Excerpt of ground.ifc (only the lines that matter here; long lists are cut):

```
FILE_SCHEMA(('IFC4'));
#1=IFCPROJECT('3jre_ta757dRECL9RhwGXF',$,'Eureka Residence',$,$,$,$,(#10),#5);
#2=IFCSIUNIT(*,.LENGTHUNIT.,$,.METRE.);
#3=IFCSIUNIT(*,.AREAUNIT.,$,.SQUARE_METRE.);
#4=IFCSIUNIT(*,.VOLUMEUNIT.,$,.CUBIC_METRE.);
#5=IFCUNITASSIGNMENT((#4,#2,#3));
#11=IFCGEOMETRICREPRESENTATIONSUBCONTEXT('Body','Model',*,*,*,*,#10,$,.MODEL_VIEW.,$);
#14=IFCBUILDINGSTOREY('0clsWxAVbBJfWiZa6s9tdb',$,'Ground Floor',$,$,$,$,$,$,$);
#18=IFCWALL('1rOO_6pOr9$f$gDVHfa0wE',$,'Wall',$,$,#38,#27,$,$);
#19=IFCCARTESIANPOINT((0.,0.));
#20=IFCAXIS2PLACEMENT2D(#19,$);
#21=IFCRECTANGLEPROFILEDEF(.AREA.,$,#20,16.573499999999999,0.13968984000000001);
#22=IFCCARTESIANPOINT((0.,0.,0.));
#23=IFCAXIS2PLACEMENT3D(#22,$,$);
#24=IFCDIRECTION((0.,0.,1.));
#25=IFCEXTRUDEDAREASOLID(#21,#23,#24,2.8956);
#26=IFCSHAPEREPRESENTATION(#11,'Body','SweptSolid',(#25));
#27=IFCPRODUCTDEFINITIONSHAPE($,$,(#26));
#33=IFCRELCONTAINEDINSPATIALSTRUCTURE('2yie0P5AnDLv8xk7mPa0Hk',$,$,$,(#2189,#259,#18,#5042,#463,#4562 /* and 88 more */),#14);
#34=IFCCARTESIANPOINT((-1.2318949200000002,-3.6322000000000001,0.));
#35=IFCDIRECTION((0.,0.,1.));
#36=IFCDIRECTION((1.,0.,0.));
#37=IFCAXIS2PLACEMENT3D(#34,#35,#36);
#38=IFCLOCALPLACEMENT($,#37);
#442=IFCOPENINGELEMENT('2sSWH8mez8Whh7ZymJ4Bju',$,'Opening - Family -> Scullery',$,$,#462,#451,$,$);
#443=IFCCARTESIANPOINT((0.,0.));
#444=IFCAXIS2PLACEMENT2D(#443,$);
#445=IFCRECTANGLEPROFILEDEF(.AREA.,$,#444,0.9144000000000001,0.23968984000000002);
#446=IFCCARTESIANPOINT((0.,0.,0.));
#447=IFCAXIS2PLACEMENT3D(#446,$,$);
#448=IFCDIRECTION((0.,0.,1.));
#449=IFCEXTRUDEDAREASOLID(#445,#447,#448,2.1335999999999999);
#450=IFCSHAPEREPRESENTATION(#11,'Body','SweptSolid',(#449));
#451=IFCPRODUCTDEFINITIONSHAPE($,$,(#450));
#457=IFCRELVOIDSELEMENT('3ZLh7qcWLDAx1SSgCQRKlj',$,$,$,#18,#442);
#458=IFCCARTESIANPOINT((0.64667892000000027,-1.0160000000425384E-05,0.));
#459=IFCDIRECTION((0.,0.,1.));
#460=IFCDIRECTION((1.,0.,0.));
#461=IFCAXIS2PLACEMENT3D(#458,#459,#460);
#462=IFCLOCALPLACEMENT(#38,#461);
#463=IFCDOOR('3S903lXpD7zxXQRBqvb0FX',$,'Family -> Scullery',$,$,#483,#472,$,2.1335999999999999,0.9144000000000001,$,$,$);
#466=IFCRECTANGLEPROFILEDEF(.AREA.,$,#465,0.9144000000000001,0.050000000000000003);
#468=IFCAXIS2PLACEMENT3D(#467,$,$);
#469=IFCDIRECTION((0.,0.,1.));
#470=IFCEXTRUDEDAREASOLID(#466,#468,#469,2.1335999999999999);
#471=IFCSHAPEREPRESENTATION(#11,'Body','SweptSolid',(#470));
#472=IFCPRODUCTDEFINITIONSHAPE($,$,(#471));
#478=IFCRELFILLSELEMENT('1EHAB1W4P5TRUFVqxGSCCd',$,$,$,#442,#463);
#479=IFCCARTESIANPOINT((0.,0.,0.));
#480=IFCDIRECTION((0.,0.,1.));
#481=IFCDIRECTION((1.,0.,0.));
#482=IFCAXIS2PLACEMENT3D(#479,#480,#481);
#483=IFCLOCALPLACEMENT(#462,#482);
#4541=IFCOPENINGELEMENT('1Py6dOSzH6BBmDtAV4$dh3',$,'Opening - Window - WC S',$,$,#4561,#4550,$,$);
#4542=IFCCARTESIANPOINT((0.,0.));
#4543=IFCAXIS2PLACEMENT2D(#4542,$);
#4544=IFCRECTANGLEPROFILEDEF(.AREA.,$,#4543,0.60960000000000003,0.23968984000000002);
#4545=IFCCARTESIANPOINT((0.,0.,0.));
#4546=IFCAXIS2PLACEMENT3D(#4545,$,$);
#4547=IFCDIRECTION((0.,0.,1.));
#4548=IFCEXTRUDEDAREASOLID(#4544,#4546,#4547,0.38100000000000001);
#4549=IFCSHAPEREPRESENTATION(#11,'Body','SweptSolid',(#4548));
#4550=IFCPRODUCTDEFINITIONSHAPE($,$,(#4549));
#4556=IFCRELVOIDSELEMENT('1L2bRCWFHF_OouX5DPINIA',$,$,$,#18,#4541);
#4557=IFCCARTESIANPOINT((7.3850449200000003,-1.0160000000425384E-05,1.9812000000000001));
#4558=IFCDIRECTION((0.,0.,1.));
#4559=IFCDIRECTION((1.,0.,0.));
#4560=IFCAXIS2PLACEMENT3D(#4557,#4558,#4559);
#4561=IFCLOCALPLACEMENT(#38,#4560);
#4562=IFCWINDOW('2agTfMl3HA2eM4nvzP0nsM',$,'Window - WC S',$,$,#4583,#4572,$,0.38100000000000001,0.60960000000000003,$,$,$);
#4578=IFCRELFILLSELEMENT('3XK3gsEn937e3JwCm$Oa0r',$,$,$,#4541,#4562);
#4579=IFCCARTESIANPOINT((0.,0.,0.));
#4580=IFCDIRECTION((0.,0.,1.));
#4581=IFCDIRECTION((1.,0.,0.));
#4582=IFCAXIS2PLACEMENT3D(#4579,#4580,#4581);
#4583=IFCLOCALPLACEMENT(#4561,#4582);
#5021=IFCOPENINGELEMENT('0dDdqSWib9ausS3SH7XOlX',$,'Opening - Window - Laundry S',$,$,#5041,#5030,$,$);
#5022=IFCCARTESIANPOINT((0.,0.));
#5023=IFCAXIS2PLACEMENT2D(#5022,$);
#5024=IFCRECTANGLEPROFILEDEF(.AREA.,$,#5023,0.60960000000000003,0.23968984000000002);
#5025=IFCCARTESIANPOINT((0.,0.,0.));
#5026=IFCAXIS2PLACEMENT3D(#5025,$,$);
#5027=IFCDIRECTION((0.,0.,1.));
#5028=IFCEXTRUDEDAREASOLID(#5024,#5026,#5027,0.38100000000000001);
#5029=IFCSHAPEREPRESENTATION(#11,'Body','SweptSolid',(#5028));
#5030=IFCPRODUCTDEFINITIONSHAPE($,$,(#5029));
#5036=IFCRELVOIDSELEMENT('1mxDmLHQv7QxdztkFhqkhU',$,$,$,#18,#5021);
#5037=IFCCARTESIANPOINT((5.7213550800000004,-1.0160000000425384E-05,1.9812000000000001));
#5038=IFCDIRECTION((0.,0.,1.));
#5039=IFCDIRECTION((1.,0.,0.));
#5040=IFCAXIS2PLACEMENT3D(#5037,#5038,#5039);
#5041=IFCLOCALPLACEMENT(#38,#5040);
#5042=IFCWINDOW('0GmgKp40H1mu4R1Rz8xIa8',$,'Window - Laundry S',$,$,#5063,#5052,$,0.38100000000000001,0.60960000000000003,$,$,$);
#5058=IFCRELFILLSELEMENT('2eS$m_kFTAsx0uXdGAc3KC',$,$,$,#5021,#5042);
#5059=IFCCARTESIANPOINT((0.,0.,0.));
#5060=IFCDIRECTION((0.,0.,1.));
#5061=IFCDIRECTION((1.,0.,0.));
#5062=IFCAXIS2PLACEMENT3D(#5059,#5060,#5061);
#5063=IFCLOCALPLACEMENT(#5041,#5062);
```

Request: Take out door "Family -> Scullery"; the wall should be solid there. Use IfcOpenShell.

```python
import ifcopenshell
import ifcopenshell.api.feature
import ifcopenshell.api.root
import ifcopenshell.geom
import ifcopenshell.util.shape

model = ifcopenshell.open("ground.ifc")
settings = ifcopenshell.geom.settings()


def volume(element):
    """Net volume in cubic metres, openings subtracted."""
    shape = ifcopenshell.geom.create_shape(settings, element)
    return ifcopenshell.util.shape.get_volume(shape.geometry)


door = model.by_guid("3S903lXpD7zxXQRBqvb0FX")
opening = door.FillsVoids[0].RelatingOpeningElement
wall = opening.VoidsElements[0].RelatingBuildingElement
before = volume(wall)

ifcopenshell.api.root.remove_product(model, product=door)
ifcopenshell.api.feature.remove_feature(model, feature=opening)

after = volume(wall)

print(f"wall volume {before:.3f} -> {after:.3f} m3")

model.write("ground_rev.ifc")
```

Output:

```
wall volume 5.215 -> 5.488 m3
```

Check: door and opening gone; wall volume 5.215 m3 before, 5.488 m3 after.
